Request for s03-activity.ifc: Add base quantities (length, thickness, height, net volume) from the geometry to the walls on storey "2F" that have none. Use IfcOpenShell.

First a look at what the model holds.

```python
import ifcopenshell
import ifcopenshell.util.element
import ifcopenshell.util.unit

model = ifcopenshell.open("s03-activity.ifc")
print(model.schema)
for unit_type in ("LENGTHUNIT", "AREAUNIT", "VOLUMEUNIT"):
    print(unit_type, ifcopenshell.util.unit.calculate_unit_scale(model, unit_type))
storey = next(s for s in model.by_type("IfcBuildingStorey") if s.Name == "2F")
walls = [e for e in ifcopenshell.util.element.get_decomposition(storey) if e.is_a("IfcWall")]
for e in sorted(walls, key=lambda e: e.id()):
    print(e.id(), e.is_a(), e.Name, list(ifcopenshell.util.element.get_psets(e, qtos_only=True)), sep=" | ")
```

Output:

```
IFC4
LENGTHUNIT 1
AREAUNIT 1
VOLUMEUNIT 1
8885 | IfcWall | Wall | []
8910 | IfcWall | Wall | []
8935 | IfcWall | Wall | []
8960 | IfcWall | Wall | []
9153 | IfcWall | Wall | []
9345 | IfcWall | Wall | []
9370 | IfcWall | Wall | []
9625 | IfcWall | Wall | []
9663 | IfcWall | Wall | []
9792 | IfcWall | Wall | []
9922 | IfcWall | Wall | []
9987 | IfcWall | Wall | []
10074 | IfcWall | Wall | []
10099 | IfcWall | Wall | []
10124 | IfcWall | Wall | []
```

```python
import ifcopenshell
import ifcopenshell.api.pset
import ifcopenshell.geom
import ifcopenshell.util.element
import ifcopenshell.util.shape
import ifcopenshell.util.unit

model = ifcopenshell.open("s03-activity.ifc")
unit_scale = ifcopenshell.util.unit.calculate_unit_scale(model)
volume_scale = ifcopenshell.util.unit.calculate_unit_scale(model, "VOLUMEUNIT")
settings = ifcopenshell.geom.settings()

storey = next(s for s in model.by_type("IfcBuildingStorey") if s.Name == "2F")
walls = [e for e in ifcopenshell.util.element.get_decomposition(storey) if e.is_a("IfcWall")]

for e in sorted(walls, key=lambda e: e.id()):
    if ifcopenshell.util.element.get_psets(e, qtos_only=True, should_inherit=False):
        continue
    # Geometry comes back in metres, in the element's own axes.
    shape = ifcopenshell.geom.create_shape(settings, e)
    values = {
        "Length": ifcopenshell.util.shape.get_x(shape.geometry) / unit_scale,
        "Width": ifcopenshell.util.shape.get_y(shape.geometry) / unit_scale,
        "Height": ifcopenshell.util.shape.get_z(shape.geometry) / unit_scale,
        "NetVolume": ifcopenshell.util.shape.get_volume(shape.geometry) / volume_scale,
    }
    qto = ifcopenshell.api.pset.add_qto(model, product=e, name="Qto_WallBaseQuantities")
    ifcopenshell.api.pset.edit_qto(model, qto=qto, properties=values)
    print(e.id(), {k: round(v, 3) for k, v in values.items()})

model.write("s03-activity_rev.ifc")
```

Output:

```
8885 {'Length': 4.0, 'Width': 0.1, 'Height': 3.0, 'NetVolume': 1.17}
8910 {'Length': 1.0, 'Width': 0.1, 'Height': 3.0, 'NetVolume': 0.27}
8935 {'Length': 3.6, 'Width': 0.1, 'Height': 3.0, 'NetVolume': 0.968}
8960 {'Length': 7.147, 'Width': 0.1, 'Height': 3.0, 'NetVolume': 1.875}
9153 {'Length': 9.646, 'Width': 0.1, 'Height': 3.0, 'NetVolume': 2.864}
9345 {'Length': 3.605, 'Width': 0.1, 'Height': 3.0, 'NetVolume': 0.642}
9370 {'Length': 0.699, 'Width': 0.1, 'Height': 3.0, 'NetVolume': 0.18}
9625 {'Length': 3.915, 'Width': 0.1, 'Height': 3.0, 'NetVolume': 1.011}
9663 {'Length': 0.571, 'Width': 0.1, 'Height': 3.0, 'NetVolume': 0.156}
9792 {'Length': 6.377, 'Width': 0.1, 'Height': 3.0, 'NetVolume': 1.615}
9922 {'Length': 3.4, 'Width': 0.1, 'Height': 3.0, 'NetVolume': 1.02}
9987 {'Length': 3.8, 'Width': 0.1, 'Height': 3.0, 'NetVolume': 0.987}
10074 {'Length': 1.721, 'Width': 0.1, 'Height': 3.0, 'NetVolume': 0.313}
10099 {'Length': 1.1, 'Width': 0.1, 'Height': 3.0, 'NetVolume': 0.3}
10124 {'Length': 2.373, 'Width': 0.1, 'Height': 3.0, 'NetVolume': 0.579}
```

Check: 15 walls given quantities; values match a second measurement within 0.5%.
